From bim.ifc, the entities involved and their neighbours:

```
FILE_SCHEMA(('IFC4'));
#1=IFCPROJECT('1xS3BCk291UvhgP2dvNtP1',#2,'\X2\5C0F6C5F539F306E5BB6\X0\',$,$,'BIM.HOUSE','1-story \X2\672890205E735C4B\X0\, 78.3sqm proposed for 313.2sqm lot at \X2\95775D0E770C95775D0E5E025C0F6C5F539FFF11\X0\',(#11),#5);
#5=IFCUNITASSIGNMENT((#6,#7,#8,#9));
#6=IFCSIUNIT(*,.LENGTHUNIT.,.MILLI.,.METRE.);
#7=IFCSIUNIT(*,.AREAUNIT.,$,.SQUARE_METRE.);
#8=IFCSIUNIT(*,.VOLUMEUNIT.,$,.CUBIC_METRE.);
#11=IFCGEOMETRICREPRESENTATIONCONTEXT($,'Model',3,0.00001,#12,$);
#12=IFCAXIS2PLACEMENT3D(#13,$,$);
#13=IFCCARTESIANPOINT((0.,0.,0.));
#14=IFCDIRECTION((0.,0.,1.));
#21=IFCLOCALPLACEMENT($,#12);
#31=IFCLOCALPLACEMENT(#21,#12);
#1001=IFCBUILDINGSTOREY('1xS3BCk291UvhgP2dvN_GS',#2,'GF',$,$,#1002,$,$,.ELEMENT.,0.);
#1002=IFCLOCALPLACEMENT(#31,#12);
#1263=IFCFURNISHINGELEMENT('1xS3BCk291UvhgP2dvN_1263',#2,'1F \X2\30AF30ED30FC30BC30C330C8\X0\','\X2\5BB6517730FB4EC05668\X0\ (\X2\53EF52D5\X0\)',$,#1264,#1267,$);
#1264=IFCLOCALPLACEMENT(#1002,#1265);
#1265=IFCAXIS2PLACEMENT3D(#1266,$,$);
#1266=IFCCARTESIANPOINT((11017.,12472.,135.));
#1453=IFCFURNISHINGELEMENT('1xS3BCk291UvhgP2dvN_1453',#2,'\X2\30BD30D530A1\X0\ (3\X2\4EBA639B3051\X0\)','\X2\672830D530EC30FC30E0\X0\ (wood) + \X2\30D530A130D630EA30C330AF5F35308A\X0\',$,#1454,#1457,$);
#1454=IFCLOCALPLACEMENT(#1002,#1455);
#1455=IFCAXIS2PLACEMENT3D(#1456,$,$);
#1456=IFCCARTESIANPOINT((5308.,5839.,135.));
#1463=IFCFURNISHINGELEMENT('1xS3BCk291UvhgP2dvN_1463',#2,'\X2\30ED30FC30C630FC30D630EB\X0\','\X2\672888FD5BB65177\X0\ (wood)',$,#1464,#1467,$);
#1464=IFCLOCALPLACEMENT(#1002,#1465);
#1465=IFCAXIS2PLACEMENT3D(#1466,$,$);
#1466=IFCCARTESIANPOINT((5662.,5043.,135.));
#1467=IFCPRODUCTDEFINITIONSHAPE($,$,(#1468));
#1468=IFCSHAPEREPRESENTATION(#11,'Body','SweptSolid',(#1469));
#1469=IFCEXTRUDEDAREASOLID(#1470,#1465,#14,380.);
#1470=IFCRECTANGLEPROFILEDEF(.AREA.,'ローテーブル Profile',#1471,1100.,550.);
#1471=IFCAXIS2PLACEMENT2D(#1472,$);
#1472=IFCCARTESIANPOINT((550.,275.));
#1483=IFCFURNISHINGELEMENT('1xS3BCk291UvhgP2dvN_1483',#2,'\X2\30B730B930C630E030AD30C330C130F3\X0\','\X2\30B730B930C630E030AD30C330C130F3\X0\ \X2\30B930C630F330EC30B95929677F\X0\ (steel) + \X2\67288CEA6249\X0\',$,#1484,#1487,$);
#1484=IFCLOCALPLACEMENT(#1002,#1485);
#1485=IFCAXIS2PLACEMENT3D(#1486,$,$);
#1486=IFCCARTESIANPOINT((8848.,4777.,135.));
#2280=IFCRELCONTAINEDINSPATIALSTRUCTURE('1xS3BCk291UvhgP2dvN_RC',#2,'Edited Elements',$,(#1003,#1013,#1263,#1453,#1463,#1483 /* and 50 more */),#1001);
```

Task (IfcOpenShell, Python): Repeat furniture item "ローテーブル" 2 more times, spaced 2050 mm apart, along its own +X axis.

```python
import ifcopenshell
import ifcopenshell.api.geometry
import ifcopenshell.api.root
import ifcopenshell.util.element
import ifcopenshell.util.placement
import ifcopenshell.util.unit

model = ifcopenshell.open("bim.ifc")
unit_scale = ifcopenshell.util.unit.calculate_unit_scale(model)


def reuse_history(source, copy):
    """copy_class also copies each property set's owner history, people and application; keep the originals."""
    for rel in copy.IsDefinedBy:
        if rel.is_a("IfcRelDefinesByProperties") and (history := rel.RelatingPropertyDefinition.OwnerHistory):
            rel.RelatingPropertyDefinition.OwnerHistory = source.OwnerHistory
            ifcopenshell.util.element.remove_deep2(model, history)


source = model.by_guid("1xS3BCk291UvhgP2dvN_1463")
base = ifcopenshell.util.placement.get_local_placement(source.ObjectPlacement)
step = base[:3, 0] * 2.05 / unit_scale

for i in range(1, 3):
    copy = ifcopenshell.api.root.copy_class(model, product=source)
    copy.Representation = ifcopenshell.util.element.copy_deep(
        model, source.Representation, exclude=["IfcGeometricRepresentationContext", "IfcRepresentationMap"]
    )
    reuse_history(source, copy)
    matrix = base.copy()
    matrix[:3, 3] += i * step
    print("added at", matrix[:3, 3].round(3) + 0.0)
    ifcopenshell.api.geometry.edit_object_placement(model, product=copy, matrix=matrix, is_si=False)

model.write("bim-out.ifc")
```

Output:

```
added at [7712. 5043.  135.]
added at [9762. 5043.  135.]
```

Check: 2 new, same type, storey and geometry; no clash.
